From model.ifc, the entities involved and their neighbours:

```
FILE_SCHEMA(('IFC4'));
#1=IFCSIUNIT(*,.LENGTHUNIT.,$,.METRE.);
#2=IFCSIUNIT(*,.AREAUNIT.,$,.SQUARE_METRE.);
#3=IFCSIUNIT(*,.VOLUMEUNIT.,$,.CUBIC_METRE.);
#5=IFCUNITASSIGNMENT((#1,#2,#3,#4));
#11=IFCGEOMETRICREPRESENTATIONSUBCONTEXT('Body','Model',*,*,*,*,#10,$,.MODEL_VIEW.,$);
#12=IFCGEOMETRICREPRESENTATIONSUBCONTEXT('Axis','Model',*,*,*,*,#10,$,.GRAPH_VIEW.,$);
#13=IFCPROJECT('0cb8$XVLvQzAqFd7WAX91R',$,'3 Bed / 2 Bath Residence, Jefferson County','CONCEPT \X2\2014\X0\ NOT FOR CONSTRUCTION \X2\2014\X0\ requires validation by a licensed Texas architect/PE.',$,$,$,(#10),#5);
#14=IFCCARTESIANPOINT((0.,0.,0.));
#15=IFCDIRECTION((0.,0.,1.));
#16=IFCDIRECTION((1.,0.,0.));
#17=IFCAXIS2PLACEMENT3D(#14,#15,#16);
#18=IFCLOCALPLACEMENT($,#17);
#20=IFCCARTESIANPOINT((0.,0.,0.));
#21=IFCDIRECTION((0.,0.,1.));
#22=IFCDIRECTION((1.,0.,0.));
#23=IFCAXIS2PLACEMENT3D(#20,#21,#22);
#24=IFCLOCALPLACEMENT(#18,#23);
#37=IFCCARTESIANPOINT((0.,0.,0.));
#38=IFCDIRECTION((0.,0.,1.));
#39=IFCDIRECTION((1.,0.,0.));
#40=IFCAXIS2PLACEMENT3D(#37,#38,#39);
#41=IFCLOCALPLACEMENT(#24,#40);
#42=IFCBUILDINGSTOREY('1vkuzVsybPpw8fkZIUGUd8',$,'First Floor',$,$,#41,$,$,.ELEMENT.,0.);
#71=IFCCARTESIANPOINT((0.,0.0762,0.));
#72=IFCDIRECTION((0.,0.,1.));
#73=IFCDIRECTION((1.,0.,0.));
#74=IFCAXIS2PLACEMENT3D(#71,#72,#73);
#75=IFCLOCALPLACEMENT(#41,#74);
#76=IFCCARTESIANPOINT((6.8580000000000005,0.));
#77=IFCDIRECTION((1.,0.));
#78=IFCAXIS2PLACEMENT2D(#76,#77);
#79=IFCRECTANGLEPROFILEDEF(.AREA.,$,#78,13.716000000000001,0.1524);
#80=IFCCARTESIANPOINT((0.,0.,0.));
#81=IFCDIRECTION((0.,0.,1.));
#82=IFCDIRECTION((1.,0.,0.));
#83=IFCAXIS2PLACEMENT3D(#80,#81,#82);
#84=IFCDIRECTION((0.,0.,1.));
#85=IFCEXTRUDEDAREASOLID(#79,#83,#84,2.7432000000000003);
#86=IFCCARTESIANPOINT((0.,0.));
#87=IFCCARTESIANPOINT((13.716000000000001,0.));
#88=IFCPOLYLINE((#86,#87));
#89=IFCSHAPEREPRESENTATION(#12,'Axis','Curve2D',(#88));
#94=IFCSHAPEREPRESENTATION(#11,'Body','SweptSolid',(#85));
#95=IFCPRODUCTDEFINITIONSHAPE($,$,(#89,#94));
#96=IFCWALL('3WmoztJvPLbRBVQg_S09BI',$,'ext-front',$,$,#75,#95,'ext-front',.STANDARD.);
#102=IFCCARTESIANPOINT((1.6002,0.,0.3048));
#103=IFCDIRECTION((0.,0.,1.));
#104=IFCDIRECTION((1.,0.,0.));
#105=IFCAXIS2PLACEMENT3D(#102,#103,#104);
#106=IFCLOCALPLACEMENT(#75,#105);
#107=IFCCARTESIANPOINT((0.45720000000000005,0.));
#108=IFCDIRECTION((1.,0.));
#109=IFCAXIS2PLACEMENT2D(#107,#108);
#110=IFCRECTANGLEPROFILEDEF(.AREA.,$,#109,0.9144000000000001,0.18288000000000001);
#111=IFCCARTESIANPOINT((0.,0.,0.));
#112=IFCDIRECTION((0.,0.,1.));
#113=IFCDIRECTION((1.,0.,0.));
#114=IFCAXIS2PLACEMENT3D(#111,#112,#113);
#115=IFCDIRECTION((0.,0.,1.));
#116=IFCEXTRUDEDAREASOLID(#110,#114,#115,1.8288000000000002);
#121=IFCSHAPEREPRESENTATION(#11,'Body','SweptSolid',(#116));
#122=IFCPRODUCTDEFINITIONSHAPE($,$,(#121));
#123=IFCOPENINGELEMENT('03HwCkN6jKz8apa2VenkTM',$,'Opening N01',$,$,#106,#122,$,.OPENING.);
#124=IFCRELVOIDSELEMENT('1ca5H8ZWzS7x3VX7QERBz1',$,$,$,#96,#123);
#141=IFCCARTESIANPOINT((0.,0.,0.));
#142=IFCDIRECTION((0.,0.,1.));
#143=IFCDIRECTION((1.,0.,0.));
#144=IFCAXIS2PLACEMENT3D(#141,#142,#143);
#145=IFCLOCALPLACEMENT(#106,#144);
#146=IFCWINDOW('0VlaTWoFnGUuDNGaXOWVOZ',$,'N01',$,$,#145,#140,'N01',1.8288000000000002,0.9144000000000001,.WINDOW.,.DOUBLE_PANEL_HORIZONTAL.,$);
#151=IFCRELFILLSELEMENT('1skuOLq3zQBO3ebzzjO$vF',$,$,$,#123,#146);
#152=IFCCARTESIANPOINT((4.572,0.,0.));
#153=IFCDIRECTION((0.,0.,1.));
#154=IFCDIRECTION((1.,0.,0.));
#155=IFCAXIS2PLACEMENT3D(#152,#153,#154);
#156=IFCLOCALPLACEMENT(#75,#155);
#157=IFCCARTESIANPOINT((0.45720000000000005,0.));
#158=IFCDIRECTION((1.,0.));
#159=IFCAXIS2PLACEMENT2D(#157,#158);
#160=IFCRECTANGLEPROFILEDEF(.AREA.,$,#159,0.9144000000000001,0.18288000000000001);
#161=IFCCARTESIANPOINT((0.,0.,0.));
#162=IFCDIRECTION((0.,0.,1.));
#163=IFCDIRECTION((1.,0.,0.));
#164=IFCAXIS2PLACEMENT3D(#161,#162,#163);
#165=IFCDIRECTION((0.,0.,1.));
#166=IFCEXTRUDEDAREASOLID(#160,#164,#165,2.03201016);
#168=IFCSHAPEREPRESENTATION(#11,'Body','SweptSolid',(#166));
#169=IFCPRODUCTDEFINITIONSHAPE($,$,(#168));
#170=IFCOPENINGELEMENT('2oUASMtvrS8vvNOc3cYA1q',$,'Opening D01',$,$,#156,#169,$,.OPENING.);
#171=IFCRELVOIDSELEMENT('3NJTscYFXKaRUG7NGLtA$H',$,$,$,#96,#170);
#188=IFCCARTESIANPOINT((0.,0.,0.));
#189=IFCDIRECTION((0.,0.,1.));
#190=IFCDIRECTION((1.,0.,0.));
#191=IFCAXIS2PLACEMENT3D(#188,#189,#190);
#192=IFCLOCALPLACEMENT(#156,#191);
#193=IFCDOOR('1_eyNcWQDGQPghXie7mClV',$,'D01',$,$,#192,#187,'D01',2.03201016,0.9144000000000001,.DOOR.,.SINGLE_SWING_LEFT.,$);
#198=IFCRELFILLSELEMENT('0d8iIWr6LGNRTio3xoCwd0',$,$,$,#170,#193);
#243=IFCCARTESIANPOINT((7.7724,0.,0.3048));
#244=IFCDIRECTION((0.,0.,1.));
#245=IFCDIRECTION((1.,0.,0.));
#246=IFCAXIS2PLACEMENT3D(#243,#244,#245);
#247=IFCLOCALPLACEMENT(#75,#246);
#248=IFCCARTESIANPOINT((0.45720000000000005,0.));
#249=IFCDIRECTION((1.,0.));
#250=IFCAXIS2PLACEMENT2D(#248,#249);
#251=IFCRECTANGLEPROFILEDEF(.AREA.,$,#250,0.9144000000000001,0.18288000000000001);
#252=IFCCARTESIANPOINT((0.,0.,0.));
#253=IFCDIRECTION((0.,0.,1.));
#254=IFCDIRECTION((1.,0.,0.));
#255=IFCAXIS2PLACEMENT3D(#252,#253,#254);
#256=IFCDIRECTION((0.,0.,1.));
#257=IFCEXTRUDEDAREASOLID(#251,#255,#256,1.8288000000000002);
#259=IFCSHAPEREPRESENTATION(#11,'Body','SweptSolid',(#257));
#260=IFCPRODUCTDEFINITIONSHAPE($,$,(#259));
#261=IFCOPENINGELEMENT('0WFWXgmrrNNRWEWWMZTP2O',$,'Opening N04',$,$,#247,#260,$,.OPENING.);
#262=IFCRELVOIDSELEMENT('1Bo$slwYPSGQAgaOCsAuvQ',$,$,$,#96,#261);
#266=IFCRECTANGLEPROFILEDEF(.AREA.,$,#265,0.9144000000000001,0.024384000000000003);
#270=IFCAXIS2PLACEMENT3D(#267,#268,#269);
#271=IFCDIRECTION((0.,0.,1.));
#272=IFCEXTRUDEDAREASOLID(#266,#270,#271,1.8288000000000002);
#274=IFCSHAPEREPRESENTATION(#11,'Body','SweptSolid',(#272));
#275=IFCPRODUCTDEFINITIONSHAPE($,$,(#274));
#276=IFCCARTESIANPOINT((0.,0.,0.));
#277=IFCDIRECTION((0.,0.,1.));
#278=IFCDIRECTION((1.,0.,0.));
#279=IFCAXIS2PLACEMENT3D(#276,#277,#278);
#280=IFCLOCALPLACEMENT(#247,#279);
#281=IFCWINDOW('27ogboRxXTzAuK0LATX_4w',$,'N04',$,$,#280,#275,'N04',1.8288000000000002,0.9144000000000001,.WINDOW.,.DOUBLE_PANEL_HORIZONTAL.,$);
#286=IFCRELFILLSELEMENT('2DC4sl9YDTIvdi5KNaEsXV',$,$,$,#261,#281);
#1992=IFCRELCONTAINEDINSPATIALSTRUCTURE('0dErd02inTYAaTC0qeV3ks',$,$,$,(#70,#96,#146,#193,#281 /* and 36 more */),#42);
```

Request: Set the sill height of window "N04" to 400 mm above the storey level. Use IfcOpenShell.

```python
import numpy as np
import ifcopenshell
import ifcopenshell.api.geometry
import ifcopenshell.geom
import ifcopenshell.util.element
import ifcopenshell.util.placement
import ifcopenshell.util.shape
import ifcopenshell.util.unit

model = ifcopenshell.open("model.ifc")
unit_scale = ifcopenshell.util.unit.calculate_unit_scale(model)

window = model.by_guid("27ogboRxXTzAuK0LATX_4w")
opening = window.FillsVoids[0].RelatingOpeningElement
storey = ifcopenshell.util.element.get_container(window, ifc_class="IfcBuildingStorey")
level = ifcopenshell.util.placement.get_local_placement(storey.ObjectPlacement)[2, 3]

# The opening's origin need not be at the sill, so measure its lowest point.
shape = ifcopenshell.geom.create_shape(ifcopenshell.geom.settings(), opening)
bottom = ifcopenshell.util.shape.get_shape_bottom_elevation(shape, shape.geometry) / unit_scale
dz = level + 0.4 / unit_scale - bottom

shift = np.array([0.0, 0.0, dz])
# The window is placed relative to its opening, so it follows when the opening moves.
matrix = ifcopenshell.util.placement.get_local_placement(opening.ObjectPlacement)
matrix[:3, 3] += shift
ifcopenshell.api.geometry.edit_object_placement(
    model, product=opening, matrix=matrix, is_si=False, should_transform_children=True
)

print(f"moved by {dz * unit_scale:+.3f} m")

model.write("model_updated.ifc")
```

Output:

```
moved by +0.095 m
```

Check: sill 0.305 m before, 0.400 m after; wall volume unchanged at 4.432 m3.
